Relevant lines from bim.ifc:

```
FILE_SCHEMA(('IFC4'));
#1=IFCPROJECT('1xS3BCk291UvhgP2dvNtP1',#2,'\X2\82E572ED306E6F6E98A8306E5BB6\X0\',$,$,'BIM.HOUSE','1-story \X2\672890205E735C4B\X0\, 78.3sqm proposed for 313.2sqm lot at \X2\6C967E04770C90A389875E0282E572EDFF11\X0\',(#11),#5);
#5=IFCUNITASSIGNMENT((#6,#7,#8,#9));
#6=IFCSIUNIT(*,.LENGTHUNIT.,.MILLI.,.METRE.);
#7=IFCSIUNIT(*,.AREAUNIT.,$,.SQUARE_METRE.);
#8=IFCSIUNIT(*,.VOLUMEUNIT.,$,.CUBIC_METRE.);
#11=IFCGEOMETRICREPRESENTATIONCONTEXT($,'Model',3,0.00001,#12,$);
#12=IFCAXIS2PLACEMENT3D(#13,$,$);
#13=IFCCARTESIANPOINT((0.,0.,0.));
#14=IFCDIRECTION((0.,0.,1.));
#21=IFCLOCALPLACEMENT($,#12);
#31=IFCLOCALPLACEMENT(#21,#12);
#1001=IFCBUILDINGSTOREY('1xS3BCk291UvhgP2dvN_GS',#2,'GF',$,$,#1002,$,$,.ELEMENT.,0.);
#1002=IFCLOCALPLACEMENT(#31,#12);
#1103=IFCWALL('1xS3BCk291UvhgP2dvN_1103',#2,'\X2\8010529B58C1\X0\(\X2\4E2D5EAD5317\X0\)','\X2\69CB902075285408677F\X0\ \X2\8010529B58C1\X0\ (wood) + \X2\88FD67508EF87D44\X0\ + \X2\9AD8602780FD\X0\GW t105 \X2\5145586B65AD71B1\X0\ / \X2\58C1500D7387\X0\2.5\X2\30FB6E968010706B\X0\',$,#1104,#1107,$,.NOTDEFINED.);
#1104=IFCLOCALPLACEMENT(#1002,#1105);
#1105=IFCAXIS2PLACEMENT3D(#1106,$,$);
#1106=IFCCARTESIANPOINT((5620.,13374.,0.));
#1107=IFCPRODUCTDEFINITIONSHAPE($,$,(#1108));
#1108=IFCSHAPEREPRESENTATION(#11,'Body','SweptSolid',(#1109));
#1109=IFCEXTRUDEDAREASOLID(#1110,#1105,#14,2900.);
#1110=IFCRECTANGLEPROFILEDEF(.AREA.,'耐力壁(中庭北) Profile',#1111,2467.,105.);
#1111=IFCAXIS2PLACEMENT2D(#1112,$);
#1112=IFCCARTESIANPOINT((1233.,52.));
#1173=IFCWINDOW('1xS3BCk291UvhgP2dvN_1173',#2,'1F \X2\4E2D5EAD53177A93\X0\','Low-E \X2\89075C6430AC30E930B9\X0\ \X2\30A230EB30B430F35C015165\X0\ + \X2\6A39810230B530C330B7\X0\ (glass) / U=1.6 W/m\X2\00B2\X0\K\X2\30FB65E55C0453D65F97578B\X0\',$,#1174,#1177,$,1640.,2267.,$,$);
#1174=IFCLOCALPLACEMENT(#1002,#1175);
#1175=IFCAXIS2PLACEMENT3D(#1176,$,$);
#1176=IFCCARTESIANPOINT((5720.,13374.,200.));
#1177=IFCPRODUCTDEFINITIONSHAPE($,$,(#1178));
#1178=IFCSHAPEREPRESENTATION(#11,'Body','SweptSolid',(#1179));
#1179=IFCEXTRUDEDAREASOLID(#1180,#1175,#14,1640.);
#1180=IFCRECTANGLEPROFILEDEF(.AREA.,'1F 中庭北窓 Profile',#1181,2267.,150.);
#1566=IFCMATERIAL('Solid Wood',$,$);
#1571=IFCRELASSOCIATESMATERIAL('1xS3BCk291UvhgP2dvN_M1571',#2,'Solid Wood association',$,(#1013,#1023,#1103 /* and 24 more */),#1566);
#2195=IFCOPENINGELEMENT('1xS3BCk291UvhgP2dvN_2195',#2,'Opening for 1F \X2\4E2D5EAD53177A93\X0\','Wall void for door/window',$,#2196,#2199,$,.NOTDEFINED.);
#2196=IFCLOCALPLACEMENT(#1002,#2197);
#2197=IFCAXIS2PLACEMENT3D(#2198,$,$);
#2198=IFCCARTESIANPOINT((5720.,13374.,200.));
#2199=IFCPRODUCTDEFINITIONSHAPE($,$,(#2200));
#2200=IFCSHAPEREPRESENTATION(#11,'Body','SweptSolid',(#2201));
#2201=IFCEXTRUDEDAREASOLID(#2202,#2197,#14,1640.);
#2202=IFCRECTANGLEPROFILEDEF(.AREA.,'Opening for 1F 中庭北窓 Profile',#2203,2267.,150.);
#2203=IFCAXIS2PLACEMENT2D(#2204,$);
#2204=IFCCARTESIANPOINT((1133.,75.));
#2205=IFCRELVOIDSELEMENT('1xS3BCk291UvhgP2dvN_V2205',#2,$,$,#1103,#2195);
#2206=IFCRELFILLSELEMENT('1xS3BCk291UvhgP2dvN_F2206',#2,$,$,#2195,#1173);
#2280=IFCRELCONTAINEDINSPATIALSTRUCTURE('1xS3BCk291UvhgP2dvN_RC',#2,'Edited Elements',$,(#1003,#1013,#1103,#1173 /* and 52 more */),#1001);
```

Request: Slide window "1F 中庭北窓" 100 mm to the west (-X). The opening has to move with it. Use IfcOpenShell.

```python
import ifcopenshell
import ifcopenshell.api.geometry
import ifcopenshell.util.placement
import ifcopenshell.util.unit

model = ifcopenshell.open("bim.ifc")
unit_scale = ifcopenshell.util.unit.calculate_unit_scale(model)

window = model.by_guid("1xS3BCk291UvhgP2dvN_1173")
opening = window.FillsVoids[0].RelatingOpeningElement
wall = opening.VoidsElements[0].RelatingBuildingElement

wall_matrix = ifcopenshell.util.placement.get_local_placement(wall.ObjectPlacement)
shift = wall_matrix[:3, 0] * -0.1 / unit_scale
before = ifcopenshell.util.placement.get_local_placement(window.ObjectPlacement)[:3, 3].copy()

# The window is not placed relative to its opening, so move both.
for product in (opening, window):
    matrix = ifcopenshell.util.placement.get_local_placement(product.ObjectPlacement)
    matrix[:3, 3] += shift
    ifcopenshell.api.geometry.edit_object_placement(model, product=product, matrix=matrix, is_si=False)

after = ifcopenshell.util.placement.get_local_placement(window.ObjectPlacement)[:3, 3]
print("window moved by", (after - before).round(3) + 0.0)

model.write("bim_rev.ifc")
```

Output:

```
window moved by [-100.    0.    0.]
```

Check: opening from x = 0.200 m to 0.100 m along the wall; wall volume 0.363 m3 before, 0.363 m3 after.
